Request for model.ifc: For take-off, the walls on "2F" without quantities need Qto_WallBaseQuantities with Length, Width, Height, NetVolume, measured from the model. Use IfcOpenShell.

First a look at what the model holds.

```python
import ifcopenshell
import ifcopenshell.util.element
import ifcopenshell.util.unit

model = ifcopenshell.open("model.ifc")
print(model.schema)
for unit_type in ("LENGTHUNIT", "AREAUNIT", "VOLUMEUNIT"):
    print(unit_type, ifcopenshell.util.unit.calculate_unit_scale(model, unit_type))
storey = next(s for s in model.by_type("IfcBuildingStorey") if s.Name == "2F")
walls = [e for e in ifcopenshell.util.element.get_decomposition(storey) if e.is_a("IfcWall")]
for e in sorted(walls, key=lambda e: e.id()):
    print(e.id(), e.is_a(), e.Name, list(ifcopenshell.util.element.get_psets(e, qtos_only=True)), sep=" | ")
```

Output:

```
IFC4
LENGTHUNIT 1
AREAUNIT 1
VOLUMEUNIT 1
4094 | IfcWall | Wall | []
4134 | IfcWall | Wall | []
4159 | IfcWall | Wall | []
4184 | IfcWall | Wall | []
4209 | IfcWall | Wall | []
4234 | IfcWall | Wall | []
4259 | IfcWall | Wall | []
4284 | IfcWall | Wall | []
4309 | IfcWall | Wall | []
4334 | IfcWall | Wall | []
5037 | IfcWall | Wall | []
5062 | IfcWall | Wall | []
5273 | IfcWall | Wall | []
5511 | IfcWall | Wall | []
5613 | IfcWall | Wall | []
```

```python
import ifcopenshell
import ifcopenshell.api.pset
import ifcopenshell.geom
import ifcopenshell.util.element
import ifcopenshell.util.shape
import ifcopenshell.util.unit

model = ifcopenshell.open("model.ifc")
unit_scale = ifcopenshell.util.unit.calculate_unit_scale(model)
volume_scale = ifcopenshell.util.unit.calculate_unit_scale(model, "VOLUMEUNIT")
settings = ifcopenshell.geom.settings()

storey = next(s for s in model.by_type("IfcBuildingStorey") if s.Name == "2F")
walls = [e for e in ifcopenshell.util.element.get_decomposition(storey) if e.is_a("IfcWall")]

for e in sorted(walls, key=lambda e: e.id()):
    if ifcopenshell.util.element.get_psets(e, qtos_only=True, should_inherit=False):
        continue
    # Geometry comes back in metres, in the element's own axes.
    shape = ifcopenshell.geom.create_shape(settings, e)
    values = {
        "Length": ifcopenshell.util.shape.get_x(shape.geometry) / unit_scale,
        "Width": ifcopenshell.util.shape.get_y(shape.geometry) / unit_scale,
        "Height": ifcopenshell.util.shape.get_z(shape.geometry) / unit_scale,
        "NetVolume": ifcopenshell.util.shape.get_volume(shape.geometry) / volume_scale,
    }
    qto = ifcopenshell.api.pset.add_qto(model, product=e, name="Qto_WallBaseQuantities")
    ifcopenshell.api.pset.edit_qto(model, qto=qto, properties=values)
    print(e.id(), {k: round(v, 3) for k, v in values.items()})

model.write("model_v2.ifc")
```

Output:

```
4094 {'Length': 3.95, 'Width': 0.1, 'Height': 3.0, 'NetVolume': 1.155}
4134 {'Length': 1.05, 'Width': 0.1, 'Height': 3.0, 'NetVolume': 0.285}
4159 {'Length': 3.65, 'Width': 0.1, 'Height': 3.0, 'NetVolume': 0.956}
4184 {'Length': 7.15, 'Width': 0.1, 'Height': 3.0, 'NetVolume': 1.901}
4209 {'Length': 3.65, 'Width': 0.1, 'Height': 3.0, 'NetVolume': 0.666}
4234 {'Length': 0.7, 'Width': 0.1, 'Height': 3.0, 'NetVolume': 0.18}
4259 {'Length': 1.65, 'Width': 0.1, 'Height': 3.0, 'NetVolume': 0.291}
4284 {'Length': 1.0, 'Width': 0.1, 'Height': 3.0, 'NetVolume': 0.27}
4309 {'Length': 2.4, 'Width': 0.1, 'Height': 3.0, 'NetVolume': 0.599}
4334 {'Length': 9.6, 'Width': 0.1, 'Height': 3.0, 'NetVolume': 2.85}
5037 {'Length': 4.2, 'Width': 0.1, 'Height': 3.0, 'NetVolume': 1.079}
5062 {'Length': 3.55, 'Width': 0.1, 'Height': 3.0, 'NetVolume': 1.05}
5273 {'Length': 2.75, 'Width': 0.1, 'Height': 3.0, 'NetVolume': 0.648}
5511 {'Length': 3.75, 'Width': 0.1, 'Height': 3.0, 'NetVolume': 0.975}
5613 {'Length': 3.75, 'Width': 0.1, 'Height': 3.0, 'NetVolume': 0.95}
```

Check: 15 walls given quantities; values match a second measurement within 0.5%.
